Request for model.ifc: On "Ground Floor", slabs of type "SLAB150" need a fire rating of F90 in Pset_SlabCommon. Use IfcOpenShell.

First a look at what the model holds.

```python
import ifcopenshell
import ifcopenshell.util.element

model = ifcopenshell.open("model.ifc")
print(model.schema)
storey = next(s for s in model.by_type("IfcBuildingStorey") if s.Name == "Ground Floor")
slabs = [e for e in ifcopenshell.util.element.get_decomposition(storey) if e.is_a("IfcSlab")]
seen = {}
for e in slabs:
    element_type = ifcopenshell.util.element.get_type(e)
    key = (element_type.Name if element_type != e and element_type else None, ifcopenshell.util.element.get_pset(e, "Pset_SlabCommon", "FireRating"))
    seen[key] = seen.get(key, 0) + 1
for (name, value), count in sorted(seen.items(), key=str):
    print(count, "x", name, "|", value)
```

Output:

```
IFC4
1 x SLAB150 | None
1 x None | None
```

```python
import ifcopenshell
import ifcopenshell.api.pset
import ifcopenshell.util.element

model = ifcopenshell.open("model.ifc")

storey = next(s for s in model.by_type("IfcBuildingStorey") if s.Name == "Ground Floor")
slabs = [e for e in ifcopenshell.util.element.get_decomposition(storey) if e.is_a("IfcSlab")]

count = 0
for e in slabs:
    element_type = ifcopenshell.util.element.get_type(e)
    if element_type in (None, e) or element_type.Name != "SLAB150":
        continue
    # add_pset returns the element's existing set when there is one.
    pset = ifcopenshell.api.pset.add_pset(model, product=e, name="Pset_SlabCommon")
    ifcopenshell.api.pset.edit_pset(model, pset=pset, properties={"FireRating": "F90"})
    count += 1

print(count, "slabs updated")

model.write("model-out.ifc")
```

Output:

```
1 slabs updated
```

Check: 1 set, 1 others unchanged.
